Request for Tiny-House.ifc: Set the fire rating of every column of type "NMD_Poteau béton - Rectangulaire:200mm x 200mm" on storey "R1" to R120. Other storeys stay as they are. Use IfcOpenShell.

First a look at what the model holds.

```python
import ifcopenshell
import ifcopenshell.util.element

model = ifcopenshell.open("Tiny-House.ifc")
print(model.schema)
storey = next(s for s in model.by_type("IfcBuildingStorey") if s.Name == "R1")
columns = [e for e in ifcopenshell.util.element.get_decomposition(storey) if e.is_a("IfcColumn")]
seen = {}
for e in columns:
    element_type = ifcopenshell.util.element.get_type(e)
    key = (element_type.Name if element_type != e and element_type else None, ifcopenshell.util.element.get_pset(e, "Pset_ColumnCommon", "FireRating"))
    seen[key] = seen.get(key, 0) + 1
for (name, value), count in sorted(seen.items(), key=str):
    print(count, "x", name, "|", value)
```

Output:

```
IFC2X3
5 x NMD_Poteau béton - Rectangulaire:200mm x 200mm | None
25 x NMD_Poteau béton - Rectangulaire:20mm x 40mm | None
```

```python
import ifcopenshell
import ifcopenshell.api.pset
import ifcopenshell.util.element

model = ifcopenshell.open("Tiny-House.ifc")

storey = next(s for s in model.by_type("IfcBuildingStorey") if s.Name == "R1")
columns = [e for e in ifcopenshell.util.element.get_decomposition(storey) if e.is_a("IfcColumn")]

count = 0
for e in columns:
    element_type = ifcopenshell.util.element.get_type(e)
    if element_type in (None, e) or element_type.Name != "NMD_Poteau béton - Rectangulaire:200mm x 200mm":
        continue
    # add_pset returns the element's existing set when there is one.
    pset = ifcopenshell.api.pset.add_pset(model, product=e, name="Pset_ColumnCommon")
    ifcopenshell.api.pset.edit_pset(model, pset=pset, properties={"FireRating": "R120"})
    count += 1

print(count, "columns updated")

model.write("Tiny-House-out.ifc")
```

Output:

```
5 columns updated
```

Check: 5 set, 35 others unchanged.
